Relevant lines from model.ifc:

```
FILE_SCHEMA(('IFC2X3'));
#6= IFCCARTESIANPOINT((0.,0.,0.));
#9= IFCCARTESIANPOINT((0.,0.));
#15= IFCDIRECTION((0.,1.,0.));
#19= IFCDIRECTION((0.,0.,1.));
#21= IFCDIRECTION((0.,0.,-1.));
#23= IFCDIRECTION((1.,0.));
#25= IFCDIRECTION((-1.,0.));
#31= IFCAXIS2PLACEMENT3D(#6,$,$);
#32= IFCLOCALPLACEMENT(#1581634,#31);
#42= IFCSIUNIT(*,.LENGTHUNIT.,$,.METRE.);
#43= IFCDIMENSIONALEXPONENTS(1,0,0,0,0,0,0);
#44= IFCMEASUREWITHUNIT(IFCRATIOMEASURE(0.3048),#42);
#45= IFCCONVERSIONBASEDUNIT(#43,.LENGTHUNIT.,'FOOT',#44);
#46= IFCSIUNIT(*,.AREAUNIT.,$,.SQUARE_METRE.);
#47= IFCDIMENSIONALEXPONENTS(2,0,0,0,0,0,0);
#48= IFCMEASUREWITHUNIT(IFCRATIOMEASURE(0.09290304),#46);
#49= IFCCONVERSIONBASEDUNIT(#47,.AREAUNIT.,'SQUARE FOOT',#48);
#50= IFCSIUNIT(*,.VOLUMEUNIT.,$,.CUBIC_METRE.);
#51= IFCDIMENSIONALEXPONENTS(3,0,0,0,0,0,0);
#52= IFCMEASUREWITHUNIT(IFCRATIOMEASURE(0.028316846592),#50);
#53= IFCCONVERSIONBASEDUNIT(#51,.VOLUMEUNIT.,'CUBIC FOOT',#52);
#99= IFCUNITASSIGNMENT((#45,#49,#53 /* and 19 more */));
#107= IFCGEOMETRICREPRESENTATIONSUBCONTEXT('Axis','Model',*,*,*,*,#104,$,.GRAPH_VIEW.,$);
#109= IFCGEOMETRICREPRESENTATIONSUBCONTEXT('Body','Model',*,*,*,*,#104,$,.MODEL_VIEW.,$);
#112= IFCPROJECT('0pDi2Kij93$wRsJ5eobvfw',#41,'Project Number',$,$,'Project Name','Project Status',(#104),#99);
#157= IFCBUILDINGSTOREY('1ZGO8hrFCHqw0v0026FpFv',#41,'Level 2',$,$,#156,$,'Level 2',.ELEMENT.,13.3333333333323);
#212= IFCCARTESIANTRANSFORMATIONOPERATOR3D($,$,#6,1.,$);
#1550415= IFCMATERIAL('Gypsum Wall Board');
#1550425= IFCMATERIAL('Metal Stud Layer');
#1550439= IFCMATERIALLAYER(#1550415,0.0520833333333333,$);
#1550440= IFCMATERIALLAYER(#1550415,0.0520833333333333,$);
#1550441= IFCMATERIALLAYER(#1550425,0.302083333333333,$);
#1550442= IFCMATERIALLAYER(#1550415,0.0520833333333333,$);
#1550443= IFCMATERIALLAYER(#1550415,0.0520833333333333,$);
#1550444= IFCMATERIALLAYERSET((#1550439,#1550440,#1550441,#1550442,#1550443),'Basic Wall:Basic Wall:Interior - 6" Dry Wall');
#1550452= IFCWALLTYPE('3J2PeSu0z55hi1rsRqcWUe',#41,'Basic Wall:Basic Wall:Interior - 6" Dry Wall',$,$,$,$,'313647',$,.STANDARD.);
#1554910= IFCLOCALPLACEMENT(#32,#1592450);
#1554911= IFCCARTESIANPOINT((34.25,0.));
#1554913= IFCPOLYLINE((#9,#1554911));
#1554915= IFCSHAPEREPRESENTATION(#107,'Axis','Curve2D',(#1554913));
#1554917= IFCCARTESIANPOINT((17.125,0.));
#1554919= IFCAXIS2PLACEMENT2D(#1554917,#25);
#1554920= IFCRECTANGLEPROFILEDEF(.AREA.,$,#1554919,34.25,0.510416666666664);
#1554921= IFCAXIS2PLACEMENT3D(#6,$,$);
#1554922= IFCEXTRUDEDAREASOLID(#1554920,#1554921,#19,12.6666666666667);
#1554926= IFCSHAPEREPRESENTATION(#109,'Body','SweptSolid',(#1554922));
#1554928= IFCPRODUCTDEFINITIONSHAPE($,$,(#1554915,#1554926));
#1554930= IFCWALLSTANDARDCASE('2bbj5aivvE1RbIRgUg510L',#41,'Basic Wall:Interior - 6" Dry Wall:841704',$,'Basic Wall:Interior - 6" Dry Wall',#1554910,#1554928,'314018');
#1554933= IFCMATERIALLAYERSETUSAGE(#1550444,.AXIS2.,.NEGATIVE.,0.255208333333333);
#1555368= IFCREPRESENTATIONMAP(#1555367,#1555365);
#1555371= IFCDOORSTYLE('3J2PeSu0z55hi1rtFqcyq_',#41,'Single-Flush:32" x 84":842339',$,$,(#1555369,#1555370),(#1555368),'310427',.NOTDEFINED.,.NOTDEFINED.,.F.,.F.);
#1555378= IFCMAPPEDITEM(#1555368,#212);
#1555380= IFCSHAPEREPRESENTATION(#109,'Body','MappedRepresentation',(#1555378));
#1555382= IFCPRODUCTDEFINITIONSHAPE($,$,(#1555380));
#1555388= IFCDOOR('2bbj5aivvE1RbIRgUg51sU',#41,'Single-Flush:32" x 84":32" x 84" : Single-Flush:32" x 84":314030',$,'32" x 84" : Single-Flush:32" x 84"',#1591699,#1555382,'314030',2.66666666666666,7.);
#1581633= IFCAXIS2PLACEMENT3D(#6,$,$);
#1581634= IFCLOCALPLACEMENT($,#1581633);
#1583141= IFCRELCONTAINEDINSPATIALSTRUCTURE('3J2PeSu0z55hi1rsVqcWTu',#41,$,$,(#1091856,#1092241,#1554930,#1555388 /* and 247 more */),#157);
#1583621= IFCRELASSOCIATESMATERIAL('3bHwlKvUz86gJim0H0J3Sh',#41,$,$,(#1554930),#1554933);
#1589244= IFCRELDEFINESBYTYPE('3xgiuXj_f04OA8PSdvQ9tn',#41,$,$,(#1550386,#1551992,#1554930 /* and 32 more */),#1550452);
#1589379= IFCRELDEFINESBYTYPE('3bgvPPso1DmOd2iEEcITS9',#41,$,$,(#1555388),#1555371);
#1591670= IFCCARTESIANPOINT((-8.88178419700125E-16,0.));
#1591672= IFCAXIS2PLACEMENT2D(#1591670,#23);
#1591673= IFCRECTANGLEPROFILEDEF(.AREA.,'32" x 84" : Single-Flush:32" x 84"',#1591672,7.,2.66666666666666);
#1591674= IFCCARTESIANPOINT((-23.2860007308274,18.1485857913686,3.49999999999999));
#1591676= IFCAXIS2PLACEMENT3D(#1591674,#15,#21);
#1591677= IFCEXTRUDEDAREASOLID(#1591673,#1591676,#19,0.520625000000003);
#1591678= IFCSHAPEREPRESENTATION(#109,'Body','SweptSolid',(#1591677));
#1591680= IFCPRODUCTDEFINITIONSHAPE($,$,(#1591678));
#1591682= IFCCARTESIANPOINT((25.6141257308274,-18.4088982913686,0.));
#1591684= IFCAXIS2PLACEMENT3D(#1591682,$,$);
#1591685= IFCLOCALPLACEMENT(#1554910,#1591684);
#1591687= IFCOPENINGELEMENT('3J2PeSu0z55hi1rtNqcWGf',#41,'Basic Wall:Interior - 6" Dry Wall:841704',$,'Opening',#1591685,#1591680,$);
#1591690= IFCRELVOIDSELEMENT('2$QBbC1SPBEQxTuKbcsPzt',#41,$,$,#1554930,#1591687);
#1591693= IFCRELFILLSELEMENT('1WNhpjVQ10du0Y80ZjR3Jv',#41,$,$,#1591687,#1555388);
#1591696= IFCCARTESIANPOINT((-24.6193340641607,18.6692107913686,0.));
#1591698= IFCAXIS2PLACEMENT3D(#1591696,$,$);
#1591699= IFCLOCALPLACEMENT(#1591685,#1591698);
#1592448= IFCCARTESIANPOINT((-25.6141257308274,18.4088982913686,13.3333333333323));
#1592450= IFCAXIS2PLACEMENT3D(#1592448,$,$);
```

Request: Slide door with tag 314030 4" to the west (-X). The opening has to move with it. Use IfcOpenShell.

```python
import ifcopenshell
import ifcopenshell.api.geometry
import ifcopenshell.util.placement
import ifcopenshell.util.unit

model = ifcopenshell.open("model.ifc")
unit_scale = ifcopenshell.util.unit.calculate_unit_scale(model)

door = model.by_guid("2bbj5aivvE1RbIRgUg51sU")
opening = door.FillsVoids[0].RelatingOpeningElement
wall = opening.VoidsElements[0].RelatingBuildingElement

wall_matrix = ifcopenshell.util.placement.get_local_placement(wall.ObjectPlacement)
shift = wall_matrix[:3, 0] * -4 * 0.0254 / unit_scale
before = ifcopenshell.util.placement.get_local_placement(door.ObjectPlacement)[:3, 3].copy()

# The door is placed relative to its opening, so it follows when the opening moves.
matrix = ifcopenshell.util.placement.get_local_placement(opening.ObjectPlacement)
matrix[:3, 3] += shift
ifcopenshell.api.geometry.edit_object_placement(
    model, product=opening, matrix=matrix, is_si=False, should_transform_children=True
)

after = ifcopenshell.util.placement.get_local_placement(door.ObjectPlacement)[:3, 3]
print("door moved by", (after - before).round(3) + 0.0)

model.write("model-out.ifc")
```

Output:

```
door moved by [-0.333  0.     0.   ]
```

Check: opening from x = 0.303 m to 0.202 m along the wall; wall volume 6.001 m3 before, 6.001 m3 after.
